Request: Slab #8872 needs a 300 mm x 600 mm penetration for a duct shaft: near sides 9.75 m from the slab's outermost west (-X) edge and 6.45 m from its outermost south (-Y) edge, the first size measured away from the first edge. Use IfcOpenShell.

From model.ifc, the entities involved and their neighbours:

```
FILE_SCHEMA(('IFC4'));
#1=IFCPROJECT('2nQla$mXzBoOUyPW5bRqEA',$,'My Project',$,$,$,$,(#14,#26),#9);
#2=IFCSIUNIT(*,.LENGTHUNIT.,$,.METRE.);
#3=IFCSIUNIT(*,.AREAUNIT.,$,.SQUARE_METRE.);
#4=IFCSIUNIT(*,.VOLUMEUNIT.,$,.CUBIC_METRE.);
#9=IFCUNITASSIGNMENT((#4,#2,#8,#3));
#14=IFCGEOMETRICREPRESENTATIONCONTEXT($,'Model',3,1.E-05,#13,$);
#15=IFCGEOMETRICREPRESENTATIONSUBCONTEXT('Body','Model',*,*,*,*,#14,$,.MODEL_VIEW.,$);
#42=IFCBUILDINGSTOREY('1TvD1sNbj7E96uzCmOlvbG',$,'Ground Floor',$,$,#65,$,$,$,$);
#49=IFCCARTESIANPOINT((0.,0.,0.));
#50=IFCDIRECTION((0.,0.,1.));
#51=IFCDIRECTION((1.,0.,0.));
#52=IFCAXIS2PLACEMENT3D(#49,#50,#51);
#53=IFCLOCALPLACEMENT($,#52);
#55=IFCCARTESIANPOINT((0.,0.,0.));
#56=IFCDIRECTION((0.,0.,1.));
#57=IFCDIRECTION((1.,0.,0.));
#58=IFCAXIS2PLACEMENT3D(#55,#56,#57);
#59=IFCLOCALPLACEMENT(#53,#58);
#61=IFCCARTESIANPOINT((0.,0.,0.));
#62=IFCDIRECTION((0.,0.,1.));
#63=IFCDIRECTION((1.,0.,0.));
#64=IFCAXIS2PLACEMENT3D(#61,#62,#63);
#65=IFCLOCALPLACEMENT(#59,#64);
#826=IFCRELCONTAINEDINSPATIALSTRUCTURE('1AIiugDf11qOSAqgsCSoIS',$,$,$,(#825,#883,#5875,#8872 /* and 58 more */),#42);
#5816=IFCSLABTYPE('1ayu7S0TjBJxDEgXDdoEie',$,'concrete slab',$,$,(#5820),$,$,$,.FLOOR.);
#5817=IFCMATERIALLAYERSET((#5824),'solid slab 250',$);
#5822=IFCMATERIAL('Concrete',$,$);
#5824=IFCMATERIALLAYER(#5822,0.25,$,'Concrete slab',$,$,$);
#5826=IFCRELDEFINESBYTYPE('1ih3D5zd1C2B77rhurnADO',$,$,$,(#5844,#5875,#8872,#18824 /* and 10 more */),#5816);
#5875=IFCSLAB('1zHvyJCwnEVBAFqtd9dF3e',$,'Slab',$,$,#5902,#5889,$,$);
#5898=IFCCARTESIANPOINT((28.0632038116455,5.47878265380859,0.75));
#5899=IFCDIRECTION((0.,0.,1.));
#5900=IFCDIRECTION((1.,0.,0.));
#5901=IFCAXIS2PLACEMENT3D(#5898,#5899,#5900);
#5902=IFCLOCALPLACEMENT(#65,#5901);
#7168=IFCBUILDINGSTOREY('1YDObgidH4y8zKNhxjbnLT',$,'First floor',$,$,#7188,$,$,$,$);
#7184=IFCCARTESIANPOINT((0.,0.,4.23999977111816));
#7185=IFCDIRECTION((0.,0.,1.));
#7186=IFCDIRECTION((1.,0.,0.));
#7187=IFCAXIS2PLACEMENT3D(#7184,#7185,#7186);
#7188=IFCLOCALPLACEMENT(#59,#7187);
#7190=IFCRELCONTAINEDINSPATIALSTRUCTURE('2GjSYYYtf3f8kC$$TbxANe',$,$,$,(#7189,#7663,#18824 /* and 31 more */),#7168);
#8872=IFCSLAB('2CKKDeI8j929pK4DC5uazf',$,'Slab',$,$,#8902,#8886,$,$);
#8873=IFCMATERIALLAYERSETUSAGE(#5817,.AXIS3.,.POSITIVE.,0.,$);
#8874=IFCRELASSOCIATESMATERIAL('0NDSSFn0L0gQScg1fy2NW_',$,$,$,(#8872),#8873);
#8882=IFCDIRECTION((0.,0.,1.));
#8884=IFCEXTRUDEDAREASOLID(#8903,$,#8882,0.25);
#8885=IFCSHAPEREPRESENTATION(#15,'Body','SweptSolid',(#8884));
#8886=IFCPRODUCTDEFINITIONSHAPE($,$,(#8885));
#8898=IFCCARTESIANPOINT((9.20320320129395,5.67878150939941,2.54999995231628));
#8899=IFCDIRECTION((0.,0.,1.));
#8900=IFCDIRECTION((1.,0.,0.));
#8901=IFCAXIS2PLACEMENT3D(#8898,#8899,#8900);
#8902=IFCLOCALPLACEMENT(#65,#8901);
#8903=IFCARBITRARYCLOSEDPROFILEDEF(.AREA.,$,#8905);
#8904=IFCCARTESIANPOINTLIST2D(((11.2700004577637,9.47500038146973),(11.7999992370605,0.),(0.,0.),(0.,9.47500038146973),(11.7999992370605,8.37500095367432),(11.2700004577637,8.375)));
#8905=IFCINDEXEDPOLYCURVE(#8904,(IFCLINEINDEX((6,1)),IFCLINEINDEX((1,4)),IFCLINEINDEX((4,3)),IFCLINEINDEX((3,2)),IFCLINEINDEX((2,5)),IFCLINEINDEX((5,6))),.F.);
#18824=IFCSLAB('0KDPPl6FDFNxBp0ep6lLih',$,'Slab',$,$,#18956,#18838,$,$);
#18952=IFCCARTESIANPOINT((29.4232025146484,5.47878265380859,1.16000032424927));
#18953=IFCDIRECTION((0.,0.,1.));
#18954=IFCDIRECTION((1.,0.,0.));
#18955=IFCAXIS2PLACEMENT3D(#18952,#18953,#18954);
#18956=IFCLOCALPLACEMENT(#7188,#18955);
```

```python
import numpy as np
import ifcopenshell
import ifcopenshell.api.feature
import ifcopenshell.api.geometry
import ifcopenshell.api.root
import ifcopenshell.geom
import ifcopenshell.util.placement
import ifcopenshell.util.representation
import ifcopenshell.util.shape
import ifcopenshell.util.unit

model = ifcopenshell.open("model.ifc")
unit_scale = ifcopenshell.util.unit.calculate_unit_scale(model)
settings = ifcopenshell.geom.settings()


def volume(element):
    """Net volume in cubic metres, openings subtracted."""
    shape = ifcopenshell.geom.create_shape(settings, element)
    return ifcopenshell.util.shape.get_volume(shape.geometry)


slab = model.by_id(8872)
before = volume(slab)

# Extent in the slab's own axes, in metres. The edges named are its -X and -Y sides.
slab_shape = ifcopenshell.geom.create_shape(settings, slab)
vertices = ifcopenshell.util.shape.get_vertices(slab_shape.geometry)
x_min, y_min, bottom = vertices.min(axis=0)
top = vertices[:, 2].max()

opening = ifcopenshell.api.root.create_entity(model, ifc_class="IfcOpeningElement", name="Duct shaft opening", predefined_type="OPENING")
context = ifcopenshell.util.representation.get_context(model, "Model", "Body", "MODEL_VIEW")
width, depth = 0.3, 0.6
outline = [(0.0, 0.0), (width, 0.0), (width, depth), (0.0, depth), (0.0, 0.0)]
# Overshoot both faces by 50 mm so the cut is clean.
shape = ifcopenshell.api.geometry.add_slab_representation(
    model, context=context, depth=top - bottom + 0.1, polyline=outline
)
ifcopenshell.api.geometry.assign_representation(model, product=opening, representation=shape)

matrix = ifcopenshell.util.placement.get_local_placement(slab.ObjectPlacement)
matrix[:, 3] = matrix @ np.append(np.array([x_min + 9.75, y_min + 6.45, bottom - 0.05]) / unit_scale, 1.0)
ifcopenshell.api.geometry.edit_object_placement(model, product=opening, matrix=matrix, is_si=False)
ifcopenshell.api.feature.add_feature(model, feature=opening, element=slab)

after = volume(slab)

print(f"slab volume {before:.3f} -> {after:.3f} m3")

model.write("model-out.ifc")
```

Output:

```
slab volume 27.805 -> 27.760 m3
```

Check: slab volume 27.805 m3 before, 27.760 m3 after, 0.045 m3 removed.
